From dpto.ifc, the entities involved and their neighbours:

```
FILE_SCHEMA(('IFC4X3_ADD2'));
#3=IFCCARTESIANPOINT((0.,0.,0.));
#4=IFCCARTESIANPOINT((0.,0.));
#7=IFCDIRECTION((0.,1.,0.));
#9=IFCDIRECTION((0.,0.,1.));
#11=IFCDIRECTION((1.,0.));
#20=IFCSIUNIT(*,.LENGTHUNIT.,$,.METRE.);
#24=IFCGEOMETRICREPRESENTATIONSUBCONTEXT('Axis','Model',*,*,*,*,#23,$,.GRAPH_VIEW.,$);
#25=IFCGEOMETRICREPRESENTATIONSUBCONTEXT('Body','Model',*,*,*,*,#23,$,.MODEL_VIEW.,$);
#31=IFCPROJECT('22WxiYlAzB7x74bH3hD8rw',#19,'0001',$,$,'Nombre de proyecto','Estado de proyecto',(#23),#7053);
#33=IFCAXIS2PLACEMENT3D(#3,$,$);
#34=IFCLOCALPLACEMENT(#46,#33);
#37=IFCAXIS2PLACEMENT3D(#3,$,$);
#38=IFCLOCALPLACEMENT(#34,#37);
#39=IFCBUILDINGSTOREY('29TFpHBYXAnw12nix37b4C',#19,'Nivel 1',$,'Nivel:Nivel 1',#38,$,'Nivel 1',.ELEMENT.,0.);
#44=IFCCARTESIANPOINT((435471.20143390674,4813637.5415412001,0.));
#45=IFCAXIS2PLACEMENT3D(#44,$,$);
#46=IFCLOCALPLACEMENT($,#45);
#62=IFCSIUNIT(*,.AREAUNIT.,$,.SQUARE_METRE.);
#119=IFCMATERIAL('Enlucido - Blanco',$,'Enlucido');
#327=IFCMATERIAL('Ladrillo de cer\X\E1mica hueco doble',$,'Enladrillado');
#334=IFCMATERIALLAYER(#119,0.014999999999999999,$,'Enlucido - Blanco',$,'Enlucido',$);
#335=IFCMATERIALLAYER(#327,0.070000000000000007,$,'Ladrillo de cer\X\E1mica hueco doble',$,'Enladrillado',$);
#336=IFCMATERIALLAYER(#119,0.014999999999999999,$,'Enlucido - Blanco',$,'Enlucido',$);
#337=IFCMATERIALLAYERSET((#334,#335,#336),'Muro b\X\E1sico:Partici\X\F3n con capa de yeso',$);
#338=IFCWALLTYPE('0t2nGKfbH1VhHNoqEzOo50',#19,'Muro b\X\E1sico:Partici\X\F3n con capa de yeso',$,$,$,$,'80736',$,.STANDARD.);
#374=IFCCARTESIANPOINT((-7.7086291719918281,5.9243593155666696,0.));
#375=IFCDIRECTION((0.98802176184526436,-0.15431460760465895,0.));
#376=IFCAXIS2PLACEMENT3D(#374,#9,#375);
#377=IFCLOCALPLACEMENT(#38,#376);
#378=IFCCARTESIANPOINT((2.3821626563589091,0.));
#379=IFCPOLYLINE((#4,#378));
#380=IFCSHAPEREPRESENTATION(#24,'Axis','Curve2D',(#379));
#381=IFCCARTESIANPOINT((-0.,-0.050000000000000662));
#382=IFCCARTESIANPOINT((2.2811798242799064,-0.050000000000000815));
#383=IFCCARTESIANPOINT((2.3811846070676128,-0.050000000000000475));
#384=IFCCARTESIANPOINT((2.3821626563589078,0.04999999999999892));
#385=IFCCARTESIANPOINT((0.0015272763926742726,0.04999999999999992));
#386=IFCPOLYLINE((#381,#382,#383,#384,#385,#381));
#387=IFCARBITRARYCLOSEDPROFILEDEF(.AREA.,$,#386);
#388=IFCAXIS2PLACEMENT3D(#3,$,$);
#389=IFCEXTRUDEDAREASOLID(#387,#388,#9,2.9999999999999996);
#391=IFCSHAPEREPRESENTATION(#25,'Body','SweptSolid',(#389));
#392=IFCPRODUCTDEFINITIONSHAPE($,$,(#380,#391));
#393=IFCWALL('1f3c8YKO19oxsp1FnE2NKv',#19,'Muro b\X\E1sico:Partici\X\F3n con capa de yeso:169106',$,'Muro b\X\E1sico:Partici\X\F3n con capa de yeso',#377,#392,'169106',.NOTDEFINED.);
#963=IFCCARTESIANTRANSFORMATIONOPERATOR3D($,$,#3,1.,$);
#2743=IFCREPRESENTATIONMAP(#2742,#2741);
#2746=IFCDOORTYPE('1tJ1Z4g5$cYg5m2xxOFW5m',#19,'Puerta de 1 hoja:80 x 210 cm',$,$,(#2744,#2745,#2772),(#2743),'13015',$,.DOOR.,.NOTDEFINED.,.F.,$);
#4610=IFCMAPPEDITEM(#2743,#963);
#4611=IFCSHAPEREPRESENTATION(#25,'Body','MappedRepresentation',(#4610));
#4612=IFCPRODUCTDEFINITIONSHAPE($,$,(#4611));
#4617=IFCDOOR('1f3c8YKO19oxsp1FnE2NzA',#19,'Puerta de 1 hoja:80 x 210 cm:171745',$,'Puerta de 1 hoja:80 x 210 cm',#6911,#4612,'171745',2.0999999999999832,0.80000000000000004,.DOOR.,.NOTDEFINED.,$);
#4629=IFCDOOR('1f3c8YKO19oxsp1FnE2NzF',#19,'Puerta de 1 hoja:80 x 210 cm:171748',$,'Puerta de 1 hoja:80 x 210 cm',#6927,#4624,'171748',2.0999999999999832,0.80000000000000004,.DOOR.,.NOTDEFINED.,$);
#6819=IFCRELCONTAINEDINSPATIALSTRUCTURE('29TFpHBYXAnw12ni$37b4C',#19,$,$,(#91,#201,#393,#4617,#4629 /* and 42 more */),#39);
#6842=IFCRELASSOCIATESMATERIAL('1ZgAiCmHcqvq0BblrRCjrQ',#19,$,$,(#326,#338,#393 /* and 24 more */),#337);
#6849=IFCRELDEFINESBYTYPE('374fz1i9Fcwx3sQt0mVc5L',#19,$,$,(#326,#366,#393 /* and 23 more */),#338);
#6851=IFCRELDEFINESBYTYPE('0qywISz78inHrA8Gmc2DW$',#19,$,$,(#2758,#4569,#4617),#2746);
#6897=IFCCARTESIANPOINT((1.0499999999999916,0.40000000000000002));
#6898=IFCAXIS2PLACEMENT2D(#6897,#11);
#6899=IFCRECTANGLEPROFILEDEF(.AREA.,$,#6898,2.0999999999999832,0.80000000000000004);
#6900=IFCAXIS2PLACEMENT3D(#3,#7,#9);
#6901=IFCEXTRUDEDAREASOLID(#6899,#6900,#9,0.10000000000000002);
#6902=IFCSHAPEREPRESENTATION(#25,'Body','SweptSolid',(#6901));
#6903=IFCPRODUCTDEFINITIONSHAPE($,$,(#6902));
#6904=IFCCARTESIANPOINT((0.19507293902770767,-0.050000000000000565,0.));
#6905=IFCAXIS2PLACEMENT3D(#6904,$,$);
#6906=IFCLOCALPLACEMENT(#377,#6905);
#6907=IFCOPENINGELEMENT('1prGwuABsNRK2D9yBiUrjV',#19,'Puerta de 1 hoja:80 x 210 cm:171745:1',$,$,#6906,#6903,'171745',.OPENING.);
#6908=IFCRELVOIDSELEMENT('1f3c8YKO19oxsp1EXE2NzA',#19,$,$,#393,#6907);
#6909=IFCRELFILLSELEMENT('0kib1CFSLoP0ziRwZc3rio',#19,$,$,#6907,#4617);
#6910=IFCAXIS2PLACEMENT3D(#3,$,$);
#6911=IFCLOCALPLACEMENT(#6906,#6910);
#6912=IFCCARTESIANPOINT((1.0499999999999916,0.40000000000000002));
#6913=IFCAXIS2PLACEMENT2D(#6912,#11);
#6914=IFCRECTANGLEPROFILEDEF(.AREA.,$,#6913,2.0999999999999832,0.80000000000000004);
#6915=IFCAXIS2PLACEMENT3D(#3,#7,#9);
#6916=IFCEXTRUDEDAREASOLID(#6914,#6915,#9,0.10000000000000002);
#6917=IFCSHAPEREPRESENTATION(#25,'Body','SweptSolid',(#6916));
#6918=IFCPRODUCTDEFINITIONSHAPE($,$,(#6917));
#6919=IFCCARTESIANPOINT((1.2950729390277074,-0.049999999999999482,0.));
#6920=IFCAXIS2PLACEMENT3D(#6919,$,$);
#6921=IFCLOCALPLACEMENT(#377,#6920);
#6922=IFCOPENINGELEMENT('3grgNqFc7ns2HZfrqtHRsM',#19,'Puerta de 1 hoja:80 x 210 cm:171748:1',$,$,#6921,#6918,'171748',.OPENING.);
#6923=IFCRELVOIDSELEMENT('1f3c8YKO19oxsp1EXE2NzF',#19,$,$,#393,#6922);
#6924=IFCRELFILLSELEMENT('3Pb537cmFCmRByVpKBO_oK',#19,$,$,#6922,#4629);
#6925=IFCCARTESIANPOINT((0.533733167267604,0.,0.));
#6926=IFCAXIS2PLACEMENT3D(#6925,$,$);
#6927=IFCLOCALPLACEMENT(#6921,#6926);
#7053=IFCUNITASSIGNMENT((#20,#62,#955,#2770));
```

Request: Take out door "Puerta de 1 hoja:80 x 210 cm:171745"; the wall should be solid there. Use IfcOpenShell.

```python
import ifcopenshell
import ifcopenshell.api.feature
import ifcopenshell.api.root
import ifcopenshell.geom
import ifcopenshell.util.shape

model = ifcopenshell.open("dpto.ifc")
settings = ifcopenshell.geom.settings()


def volume(element):
    """Net volume in cubic metres, openings subtracted."""
    shape = ifcopenshell.geom.create_shape(settings, element)
    return ifcopenshell.util.shape.get_volume(shape.geometry)


door = model.by_guid("1f3c8YKO19oxsp1FnE2NzA")
opening = door.FillsVoids[0].RelatingOpeningElement
wall = opening.VoidsElements[0].RelatingBuildingElement
before = volume(wall)

ifcopenshell.api.root.remove_product(model, product=door)
ifcopenshell.api.feature.remove_feature(model, feature=opening)

after = volume(wall)

print(f"wall volume {before:.3f} -> {after:.3f} m3")

model.write("dpto_v2.ifc")
```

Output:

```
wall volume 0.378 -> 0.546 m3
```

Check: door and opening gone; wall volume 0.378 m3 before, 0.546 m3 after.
